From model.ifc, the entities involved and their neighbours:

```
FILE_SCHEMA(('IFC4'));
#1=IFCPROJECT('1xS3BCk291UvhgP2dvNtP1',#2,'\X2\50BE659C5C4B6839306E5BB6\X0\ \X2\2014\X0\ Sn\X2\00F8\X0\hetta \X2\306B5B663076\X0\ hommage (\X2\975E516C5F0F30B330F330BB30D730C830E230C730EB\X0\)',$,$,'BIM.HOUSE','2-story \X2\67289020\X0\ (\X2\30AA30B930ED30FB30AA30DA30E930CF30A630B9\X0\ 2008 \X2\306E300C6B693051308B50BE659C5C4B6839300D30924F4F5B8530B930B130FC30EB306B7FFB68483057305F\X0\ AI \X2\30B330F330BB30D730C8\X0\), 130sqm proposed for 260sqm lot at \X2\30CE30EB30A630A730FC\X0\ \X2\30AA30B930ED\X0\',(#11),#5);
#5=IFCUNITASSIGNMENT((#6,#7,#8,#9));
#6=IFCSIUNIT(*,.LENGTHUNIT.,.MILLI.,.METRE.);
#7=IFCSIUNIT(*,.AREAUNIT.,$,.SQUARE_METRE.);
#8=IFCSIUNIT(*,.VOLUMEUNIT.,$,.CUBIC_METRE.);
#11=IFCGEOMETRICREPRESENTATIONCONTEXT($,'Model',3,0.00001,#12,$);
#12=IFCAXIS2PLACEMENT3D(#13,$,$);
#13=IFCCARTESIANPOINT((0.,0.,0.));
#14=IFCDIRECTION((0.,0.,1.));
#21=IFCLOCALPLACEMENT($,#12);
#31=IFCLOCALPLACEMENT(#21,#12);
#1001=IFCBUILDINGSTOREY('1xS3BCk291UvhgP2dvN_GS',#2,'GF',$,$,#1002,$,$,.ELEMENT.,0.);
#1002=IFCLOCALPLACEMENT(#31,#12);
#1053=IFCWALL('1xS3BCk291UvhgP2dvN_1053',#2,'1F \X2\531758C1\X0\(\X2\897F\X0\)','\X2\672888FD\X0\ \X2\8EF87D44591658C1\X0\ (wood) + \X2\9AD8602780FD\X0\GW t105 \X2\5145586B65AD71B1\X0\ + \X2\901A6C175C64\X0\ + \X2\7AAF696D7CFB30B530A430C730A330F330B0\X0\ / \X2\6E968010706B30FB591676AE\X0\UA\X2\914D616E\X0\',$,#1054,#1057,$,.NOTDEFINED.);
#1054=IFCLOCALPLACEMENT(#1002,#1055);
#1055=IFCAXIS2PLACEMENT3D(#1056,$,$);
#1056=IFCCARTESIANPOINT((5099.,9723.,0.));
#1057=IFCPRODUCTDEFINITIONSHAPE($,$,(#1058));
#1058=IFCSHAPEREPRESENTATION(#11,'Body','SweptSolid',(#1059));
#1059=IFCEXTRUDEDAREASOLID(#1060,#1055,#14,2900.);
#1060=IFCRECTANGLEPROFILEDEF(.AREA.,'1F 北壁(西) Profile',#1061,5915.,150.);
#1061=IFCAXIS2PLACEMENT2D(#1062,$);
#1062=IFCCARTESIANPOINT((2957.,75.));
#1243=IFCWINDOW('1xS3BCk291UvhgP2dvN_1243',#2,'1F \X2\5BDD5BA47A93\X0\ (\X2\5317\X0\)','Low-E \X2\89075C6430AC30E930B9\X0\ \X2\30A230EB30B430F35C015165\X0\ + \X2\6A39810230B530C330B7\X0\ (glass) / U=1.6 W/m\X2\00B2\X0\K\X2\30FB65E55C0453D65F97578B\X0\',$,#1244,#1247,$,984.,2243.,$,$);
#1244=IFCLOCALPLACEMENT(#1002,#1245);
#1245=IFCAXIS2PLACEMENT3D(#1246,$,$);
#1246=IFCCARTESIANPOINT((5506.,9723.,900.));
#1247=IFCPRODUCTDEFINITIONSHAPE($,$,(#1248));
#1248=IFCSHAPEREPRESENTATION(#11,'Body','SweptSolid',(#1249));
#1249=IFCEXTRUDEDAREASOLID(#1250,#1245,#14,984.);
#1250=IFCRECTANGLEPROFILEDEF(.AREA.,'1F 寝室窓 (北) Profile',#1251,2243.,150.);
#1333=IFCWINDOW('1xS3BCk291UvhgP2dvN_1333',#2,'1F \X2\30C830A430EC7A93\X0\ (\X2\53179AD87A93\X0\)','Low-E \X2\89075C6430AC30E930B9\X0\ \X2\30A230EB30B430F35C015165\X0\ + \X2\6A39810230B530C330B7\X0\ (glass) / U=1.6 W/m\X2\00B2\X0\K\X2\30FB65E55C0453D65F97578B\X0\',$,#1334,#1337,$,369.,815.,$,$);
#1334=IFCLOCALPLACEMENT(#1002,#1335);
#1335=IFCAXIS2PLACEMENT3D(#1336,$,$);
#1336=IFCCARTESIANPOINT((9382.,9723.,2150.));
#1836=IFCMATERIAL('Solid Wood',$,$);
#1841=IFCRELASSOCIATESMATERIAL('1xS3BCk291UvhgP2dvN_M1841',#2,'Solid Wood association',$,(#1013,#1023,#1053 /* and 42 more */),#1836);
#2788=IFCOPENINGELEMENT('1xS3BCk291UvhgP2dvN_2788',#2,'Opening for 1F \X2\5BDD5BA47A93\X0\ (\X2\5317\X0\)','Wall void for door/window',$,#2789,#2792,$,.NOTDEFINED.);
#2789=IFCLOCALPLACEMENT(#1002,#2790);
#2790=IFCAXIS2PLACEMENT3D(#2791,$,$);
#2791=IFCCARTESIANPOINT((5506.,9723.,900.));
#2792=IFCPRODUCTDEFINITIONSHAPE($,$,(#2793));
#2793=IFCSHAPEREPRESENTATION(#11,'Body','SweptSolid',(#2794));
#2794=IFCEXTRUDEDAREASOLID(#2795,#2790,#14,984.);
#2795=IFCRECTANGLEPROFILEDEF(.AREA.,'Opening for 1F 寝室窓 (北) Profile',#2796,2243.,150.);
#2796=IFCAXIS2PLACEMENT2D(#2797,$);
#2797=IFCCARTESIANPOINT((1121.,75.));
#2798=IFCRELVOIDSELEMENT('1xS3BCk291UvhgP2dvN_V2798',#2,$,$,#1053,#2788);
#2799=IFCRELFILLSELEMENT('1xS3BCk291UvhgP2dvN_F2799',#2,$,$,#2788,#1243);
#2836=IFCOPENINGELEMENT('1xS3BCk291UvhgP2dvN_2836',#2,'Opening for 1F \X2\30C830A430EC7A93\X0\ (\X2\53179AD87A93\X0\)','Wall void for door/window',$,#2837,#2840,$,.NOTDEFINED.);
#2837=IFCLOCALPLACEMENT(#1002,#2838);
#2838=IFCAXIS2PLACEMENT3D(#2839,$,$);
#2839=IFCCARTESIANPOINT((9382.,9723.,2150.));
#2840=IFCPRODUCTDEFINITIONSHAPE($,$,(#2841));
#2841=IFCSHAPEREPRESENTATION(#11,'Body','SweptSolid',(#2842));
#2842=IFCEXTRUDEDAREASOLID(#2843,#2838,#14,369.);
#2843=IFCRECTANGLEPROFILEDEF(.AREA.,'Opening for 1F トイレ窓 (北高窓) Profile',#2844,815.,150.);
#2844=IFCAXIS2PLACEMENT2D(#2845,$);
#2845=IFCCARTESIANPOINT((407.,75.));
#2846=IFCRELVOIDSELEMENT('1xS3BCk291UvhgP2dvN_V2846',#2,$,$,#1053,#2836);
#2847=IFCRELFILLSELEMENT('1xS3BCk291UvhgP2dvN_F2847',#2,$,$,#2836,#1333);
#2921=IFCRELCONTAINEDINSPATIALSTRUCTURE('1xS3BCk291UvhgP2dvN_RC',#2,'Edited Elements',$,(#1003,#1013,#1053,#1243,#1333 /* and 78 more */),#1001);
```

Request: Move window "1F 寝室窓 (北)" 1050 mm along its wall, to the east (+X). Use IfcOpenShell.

```python
import ifcopenshell
import ifcopenshell.api.geometry
import ifcopenshell.util.placement
import ifcopenshell.util.unit

model = ifcopenshell.open("model.ifc")
unit_scale = ifcopenshell.util.unit.calculate_unit_scale(model)

window = model.by_guid("1xS3BCk291UvhgP2dvN_1243")
opening = window.FillsVoids[0].RelatingOpeningElement
wall = opening.VoidsElements[0].RelatingBuildingElement

wall_matrix = ifcopenshell.util.placement.get_local_placement(wall.ObjectPlacement)
shift = wall_matrix[:3, 0] * 1.05 / unit_scale
before = ifcopenshell.util.placement.get_local_placement(window.ObjectPlacement)[:3, 3].copy()

# The window is not placed relative to its opening, so move both.
for product in (opening, window):
    matrix = ifcopenshell.util.placement.get_local_placement(product.ObjectPlacement)
    matrix[:3, 3] += shift
    ifcopenshell.api.geometry.edit_object_placement(model, product=product, matrix=matrix, is_si=False)

after = ifcopenshell.util.placement.get_local_placement(window.ObjectPlacement)[:3, 3]
print("window moved by", (after - before).round(3) + 0.0)

model.write("model_v2.ifc")
```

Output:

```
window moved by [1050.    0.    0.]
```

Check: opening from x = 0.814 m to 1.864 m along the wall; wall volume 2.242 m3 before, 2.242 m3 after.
